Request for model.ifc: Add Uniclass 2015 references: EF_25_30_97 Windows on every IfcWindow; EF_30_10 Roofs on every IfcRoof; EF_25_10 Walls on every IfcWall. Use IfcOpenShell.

First a look at what the model holds.

```python
import ifcopenshell

model = ifcopenshell.open("model.ifc")
print(model.schema)
print("classifications:", [c.Name for c in model.by_type("IfcClassification")])
for ifc_class in ("IfcDoor", "IfcRoof", "IfcStair", "IfcWall", "IfcWindow"):
    print(ifc_class, len(model.by_type(ifc_class)))
```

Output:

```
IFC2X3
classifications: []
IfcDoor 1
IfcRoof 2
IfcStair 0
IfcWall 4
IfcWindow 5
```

```python
import ifcopenshell
import ifcopenshell.api.classification

model = ifcopenshell.open("model.ifc")

# IFC2X3 requires Source and Edition and has no link from the project to the system.
system = model.create_entity("IfcClassification", Source="NBS", Edition="2015", Name="Uniclass 2015")

codes = {
    "IfcWindow": ("EF_25_30_97", "Windows"),
    "IfcRoof": ("EF_30_10", "Roofs"),
    "IfcWall": ("EF_25_10", "Walls"),
}
for ifc_class, (code, name) in codes.items():
    products = model.by_type(ifc_class)
    ifcopenshell.api.classification.add_reference(
        model, products=products, classification=system, identification=code, name=name
    )
    print(code, len(products))

model.write("model_v2.ifc")
```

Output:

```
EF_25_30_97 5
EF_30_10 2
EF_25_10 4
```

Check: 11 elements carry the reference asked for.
